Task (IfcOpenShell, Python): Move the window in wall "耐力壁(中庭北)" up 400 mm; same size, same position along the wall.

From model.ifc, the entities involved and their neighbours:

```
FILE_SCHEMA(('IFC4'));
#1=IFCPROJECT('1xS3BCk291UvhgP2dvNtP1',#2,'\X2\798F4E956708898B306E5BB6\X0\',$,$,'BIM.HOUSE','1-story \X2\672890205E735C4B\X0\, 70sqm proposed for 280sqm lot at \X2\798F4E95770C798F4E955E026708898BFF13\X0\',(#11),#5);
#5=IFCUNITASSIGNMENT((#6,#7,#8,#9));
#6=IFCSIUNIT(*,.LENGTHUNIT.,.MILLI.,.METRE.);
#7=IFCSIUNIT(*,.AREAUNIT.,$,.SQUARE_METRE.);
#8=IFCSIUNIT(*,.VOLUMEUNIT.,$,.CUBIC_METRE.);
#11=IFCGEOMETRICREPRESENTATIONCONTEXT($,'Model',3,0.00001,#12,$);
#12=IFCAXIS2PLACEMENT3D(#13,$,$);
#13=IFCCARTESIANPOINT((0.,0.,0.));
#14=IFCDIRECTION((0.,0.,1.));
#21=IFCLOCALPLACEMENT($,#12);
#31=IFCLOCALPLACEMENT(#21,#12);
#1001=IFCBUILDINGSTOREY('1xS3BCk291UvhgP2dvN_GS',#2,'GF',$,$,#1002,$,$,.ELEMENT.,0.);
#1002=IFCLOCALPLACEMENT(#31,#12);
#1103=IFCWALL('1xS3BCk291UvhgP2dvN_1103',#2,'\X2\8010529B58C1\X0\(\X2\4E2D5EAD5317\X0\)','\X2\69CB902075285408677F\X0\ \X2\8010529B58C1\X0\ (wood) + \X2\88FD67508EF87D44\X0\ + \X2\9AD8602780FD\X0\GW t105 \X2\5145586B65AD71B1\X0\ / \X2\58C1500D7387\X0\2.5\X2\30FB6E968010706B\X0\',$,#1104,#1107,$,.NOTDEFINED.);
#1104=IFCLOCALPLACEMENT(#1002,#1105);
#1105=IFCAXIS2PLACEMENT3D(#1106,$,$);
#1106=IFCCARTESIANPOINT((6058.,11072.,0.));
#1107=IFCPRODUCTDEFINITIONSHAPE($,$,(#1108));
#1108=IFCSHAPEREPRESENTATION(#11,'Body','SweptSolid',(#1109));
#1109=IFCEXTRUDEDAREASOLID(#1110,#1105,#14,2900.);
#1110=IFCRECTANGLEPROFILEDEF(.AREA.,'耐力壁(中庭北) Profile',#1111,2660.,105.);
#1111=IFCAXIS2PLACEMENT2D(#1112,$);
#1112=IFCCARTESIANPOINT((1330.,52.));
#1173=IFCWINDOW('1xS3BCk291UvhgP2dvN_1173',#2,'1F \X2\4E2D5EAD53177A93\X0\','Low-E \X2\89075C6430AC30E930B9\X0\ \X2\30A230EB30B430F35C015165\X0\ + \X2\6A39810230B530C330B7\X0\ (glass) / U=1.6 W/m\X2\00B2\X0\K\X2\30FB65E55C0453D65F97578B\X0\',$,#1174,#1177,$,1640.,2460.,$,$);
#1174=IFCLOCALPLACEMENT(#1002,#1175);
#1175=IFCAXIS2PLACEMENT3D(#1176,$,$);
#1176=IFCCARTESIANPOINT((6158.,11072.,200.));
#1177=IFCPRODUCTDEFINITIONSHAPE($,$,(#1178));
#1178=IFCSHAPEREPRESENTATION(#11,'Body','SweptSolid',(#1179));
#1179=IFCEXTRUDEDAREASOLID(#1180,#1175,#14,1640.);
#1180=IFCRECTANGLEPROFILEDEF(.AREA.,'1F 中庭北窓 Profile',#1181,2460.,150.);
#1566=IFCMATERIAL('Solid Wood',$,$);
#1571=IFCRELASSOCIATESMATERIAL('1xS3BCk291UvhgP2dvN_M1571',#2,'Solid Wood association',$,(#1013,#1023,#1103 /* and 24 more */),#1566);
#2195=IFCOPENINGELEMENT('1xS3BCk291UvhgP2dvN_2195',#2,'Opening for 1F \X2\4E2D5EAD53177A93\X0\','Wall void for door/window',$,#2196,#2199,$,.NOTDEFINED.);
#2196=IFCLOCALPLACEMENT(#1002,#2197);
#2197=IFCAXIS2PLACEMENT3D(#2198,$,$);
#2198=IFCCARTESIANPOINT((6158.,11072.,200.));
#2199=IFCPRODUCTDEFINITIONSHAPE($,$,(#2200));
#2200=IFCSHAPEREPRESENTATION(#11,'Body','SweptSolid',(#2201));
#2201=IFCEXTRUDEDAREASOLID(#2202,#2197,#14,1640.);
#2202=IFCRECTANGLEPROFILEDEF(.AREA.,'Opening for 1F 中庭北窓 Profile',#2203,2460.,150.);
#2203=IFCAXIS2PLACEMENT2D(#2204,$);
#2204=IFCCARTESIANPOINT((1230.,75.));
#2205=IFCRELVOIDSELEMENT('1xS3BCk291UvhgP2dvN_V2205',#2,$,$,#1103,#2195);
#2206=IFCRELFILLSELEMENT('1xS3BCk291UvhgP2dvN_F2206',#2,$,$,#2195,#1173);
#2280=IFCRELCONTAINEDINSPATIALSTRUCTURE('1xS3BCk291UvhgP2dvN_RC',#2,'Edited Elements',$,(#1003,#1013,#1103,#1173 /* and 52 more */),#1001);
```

```python
import numpy as np
import ifcopenshell
import ifcopenshell.api.geometry
import ifcopenshell.util.placement
import ifcopenshell.util.unit

model = ifcopenshell.open("model.ifc")
unit_scale = ifcopenshell.util.unit.calculate_unit_scale(model)

window = model.by_id(1173)
opening = window.FillsVoids[0].RelatingOpeningElement
dz = 400.0

shift = np.array([0.0, 0.0, dz])
# The window is not placed relative to its opening, so move both.
for product in (opening, window):
    matrix = ifcopenshell.util.placement.get_local_placement(product.ObjectPlacement)
    matrix[:3, 3] += shift
    ifcopenshell.api.geometry.edit_object_placement(model, product=product, matrix=matrix, is_si=False)

print(f"moved by {dz * unit_scale:+.3f} m")

model.write("model_updated.ifc")
```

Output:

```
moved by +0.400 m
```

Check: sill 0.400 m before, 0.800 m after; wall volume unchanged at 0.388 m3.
